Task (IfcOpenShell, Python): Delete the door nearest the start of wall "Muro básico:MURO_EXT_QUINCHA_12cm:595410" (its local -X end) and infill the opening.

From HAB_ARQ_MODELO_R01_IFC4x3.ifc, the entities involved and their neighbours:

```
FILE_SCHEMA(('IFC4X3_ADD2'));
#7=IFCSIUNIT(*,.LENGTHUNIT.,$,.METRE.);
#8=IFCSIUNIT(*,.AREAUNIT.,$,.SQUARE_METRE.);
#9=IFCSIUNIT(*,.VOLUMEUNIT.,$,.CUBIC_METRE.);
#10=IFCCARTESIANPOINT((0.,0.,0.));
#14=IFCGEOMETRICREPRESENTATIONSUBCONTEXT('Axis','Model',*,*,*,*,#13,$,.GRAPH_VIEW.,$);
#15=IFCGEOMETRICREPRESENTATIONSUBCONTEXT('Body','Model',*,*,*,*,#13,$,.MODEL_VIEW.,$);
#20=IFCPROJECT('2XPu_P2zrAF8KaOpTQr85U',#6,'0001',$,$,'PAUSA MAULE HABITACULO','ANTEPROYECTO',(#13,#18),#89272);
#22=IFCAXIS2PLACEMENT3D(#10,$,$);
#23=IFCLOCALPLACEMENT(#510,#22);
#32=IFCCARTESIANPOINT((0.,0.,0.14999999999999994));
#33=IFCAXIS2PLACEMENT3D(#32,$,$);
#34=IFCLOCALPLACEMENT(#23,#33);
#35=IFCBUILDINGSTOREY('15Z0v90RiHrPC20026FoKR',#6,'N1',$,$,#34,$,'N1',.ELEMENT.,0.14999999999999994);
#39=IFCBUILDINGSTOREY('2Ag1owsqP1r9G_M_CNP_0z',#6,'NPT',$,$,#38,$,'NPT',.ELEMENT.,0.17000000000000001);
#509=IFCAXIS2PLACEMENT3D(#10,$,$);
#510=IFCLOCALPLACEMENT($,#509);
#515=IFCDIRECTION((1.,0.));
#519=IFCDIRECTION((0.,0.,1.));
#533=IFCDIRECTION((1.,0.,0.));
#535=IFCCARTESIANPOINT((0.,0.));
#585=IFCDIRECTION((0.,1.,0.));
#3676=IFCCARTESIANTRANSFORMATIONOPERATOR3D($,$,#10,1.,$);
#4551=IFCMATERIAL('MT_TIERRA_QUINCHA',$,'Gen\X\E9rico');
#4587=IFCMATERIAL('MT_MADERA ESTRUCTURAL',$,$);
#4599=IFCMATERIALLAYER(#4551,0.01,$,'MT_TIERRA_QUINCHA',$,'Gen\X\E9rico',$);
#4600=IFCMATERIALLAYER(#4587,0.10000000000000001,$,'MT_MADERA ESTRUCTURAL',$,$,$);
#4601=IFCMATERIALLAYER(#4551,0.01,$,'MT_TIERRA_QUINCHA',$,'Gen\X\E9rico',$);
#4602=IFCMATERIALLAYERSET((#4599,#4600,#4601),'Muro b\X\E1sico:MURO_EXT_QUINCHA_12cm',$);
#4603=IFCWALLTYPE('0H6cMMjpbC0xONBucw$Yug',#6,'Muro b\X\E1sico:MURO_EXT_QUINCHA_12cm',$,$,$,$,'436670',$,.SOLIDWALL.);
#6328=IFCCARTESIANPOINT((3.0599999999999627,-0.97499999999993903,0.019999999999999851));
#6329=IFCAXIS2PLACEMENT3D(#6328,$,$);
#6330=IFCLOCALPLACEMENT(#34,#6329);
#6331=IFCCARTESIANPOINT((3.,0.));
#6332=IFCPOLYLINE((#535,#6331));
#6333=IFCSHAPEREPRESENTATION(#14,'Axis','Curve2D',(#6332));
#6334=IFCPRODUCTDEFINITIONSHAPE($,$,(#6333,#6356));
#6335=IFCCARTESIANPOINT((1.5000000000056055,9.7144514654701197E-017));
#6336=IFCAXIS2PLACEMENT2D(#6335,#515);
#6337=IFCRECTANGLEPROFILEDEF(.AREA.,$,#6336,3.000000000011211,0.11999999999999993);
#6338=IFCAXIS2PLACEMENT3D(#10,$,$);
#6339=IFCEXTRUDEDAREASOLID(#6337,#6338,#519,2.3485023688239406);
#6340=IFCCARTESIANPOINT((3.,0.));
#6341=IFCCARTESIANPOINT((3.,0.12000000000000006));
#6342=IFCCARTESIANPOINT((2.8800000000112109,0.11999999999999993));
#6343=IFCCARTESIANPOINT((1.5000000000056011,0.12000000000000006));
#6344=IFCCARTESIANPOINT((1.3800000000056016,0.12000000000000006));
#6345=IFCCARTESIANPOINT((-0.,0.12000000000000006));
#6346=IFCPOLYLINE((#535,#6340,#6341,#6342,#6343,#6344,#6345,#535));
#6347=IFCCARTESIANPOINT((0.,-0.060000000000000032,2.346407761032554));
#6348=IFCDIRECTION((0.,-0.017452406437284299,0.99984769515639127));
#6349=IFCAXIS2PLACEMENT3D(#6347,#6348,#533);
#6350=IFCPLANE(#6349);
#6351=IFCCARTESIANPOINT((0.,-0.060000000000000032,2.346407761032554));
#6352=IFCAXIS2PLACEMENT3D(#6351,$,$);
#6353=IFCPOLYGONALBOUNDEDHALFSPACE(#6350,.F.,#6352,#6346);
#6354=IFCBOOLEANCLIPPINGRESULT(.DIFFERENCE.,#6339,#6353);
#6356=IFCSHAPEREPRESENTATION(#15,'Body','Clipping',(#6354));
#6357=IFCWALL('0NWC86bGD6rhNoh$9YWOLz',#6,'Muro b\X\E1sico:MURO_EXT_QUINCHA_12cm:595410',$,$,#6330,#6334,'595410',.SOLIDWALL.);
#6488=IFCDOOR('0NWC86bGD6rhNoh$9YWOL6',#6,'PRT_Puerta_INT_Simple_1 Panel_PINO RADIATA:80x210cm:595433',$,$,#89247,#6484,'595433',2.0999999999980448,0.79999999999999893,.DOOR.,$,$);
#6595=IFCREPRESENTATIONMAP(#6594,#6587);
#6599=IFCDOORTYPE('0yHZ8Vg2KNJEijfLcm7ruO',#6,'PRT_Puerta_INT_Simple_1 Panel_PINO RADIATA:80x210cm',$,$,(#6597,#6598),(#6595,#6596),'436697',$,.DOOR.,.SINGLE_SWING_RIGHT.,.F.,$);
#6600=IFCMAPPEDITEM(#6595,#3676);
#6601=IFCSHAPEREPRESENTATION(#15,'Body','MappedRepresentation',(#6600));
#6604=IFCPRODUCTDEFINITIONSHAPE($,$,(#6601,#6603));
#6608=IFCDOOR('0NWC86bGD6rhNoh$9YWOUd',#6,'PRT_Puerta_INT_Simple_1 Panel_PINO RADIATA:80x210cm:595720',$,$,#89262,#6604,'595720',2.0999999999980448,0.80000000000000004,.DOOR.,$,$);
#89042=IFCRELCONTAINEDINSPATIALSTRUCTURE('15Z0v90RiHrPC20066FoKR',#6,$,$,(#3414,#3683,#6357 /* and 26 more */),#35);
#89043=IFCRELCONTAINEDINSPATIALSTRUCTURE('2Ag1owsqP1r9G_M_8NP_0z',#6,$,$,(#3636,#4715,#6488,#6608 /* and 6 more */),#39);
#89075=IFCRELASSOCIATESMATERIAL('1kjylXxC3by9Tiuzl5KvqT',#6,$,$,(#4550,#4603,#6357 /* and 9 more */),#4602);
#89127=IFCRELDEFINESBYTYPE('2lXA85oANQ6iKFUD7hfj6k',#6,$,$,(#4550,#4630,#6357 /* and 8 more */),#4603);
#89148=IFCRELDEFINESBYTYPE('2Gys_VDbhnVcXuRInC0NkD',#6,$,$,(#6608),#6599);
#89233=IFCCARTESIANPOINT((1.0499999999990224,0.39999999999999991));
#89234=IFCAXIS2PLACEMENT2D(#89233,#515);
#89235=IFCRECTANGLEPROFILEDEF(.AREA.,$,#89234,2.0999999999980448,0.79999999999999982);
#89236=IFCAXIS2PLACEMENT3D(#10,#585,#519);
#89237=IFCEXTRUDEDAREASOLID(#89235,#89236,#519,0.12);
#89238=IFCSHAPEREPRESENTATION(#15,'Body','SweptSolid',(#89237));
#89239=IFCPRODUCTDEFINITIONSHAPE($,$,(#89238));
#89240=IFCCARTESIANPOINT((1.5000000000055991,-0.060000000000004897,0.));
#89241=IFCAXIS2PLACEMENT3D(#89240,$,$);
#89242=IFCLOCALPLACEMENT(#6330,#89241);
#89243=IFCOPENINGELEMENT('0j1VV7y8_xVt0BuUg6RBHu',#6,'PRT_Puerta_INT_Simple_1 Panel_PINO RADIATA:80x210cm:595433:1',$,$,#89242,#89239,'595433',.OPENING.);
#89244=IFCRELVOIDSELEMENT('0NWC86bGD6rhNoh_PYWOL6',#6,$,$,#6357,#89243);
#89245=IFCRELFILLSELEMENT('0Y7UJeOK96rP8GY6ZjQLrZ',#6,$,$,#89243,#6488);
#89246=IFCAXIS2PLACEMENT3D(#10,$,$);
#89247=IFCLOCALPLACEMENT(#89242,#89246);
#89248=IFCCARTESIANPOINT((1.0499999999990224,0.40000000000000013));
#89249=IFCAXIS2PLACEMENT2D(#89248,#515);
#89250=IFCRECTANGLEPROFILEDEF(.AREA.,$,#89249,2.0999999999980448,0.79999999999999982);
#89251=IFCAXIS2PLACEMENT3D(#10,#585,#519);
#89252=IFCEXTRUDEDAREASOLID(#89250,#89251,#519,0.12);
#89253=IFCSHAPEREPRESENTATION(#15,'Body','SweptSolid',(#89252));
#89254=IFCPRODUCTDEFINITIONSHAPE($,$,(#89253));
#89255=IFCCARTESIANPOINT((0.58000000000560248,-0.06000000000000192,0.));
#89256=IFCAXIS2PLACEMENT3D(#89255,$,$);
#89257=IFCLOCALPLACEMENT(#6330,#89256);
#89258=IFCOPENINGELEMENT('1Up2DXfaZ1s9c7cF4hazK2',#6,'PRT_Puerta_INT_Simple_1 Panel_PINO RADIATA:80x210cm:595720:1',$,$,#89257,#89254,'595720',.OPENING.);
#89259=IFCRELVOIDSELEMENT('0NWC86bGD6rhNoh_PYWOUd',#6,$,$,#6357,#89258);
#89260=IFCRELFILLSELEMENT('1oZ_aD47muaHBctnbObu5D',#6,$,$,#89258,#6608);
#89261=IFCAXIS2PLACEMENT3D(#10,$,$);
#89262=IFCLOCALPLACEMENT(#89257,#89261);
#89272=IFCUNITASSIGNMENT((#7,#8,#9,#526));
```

```python
import ifcopenshell
import ifcopenshell.api.feature
import ifcopenshell.api.root
import ifcopenshell.geom
import ifcopenshell.util.shape

model = ifcopenshell.open("HAB_ARQ_MODELO_R01_IFC4x3.ifc")
settings = ifcopenshell.geom.settings()


def volume(element):
    """Net volume in cubic metres, openings subtracted."""
    shape = ifcopenshell.geom.create_shape(settings, element)
    return ifcopenshell.util.shape.get_volume(shape.geometry)


door = model.by_guid("0NWC86bGD6rhNoh$9YWOUd")
opening = door.FillsVoids[0].RelatingOpeningElement
wall = opening.VoidsElements[0].RelatingBuildingElement
before = volume(wall)

ifcopenshell.api.root.remove_product(model, product=door)
ifcopenshell.api.feature.remove_feature(model, feature=opening)

after = volume(wall)

print(f"wall volume {before:.3f} -> {after:.3f} m3")

model.write("HAB_ARQ_MODELO_R01_IFC4x3_rev.ifc")
```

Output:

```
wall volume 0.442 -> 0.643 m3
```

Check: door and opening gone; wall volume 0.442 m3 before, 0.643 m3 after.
